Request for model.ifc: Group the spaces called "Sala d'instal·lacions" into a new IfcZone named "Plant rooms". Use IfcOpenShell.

First a look at what the model holds.

```python
import ifcopenshell

model = ifcopenshell.open("model.ifc")
print(model.schema)
seen = {}
for space in model.by_type("IfcSpace"):
    seen[space.LongName] = seen.get(space.LongName, 0) + 1
for name, count in sorted(seen.items(), key=str):
    print(count, "x", name)
print("zones:", [z.Name for z in model.by_type("IfcZone")][:20])
```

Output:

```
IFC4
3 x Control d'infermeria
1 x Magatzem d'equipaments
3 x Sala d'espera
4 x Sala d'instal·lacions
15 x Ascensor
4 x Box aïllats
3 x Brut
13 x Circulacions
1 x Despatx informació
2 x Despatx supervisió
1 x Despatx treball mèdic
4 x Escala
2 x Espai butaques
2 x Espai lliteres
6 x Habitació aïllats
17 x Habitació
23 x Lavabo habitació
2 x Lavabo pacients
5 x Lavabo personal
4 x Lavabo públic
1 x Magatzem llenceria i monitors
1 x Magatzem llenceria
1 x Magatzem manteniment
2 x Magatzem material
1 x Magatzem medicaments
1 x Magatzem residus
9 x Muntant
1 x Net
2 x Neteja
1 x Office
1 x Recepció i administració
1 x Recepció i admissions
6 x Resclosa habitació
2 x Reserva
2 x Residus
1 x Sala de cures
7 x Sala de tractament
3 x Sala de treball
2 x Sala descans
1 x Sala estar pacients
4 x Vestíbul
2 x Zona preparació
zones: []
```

```python
import ifcopenshell
import ifcopenshell.api.group
import ifcopenshell.api.root

model = ifcopenshell.open("model.ifc")

names = {"Sala d'instal·lacions"}
spaces = [s for s in model.by_type("IfcSpace") if s.LongName in names]

zone = ifcopenshell.api.root.create_entity(model, ifc_class="IfcZone", name="Plant rooms")
ifcopenshell.api.group.assign_group(model, products=spaces, group=zone)
print(len(spaces), "spaces in", zone.Name)

model.write("model_v2.ifc")
```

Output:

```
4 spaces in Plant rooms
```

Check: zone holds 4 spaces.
